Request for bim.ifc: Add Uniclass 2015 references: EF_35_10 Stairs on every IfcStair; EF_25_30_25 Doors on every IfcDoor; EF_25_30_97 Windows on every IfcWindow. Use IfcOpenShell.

First a look at what the model holds.

```python
import ifcopenshell

model = ifcopenshell.open("bim.ifc")
print(model.schema)
print("classifications:", [c.Name for c in model.by_type("IfcClassification")])
for ifc_class in ("IfcDoor", "IfcRoof", "IfcStair", "IfcWall", "IfcWindow"):
    print(ifc_class, len(model.by_type(ifc_class)))
```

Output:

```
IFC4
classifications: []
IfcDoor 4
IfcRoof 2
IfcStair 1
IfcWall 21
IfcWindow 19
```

```python
import ifcopenshell
import ifcopenshell.api.classification

model = ifcopenshell.open("bim.ifc")

system = ifcopenshell.api.classification.add_classification(model, classification="Uniclass 2015")

codes = {
    "IfcStair": ("EF_35_10", "Stairs"),
    "IfcDoor": ("EF_25_30_25", "Doors"),
    "IfcWindow": ("EF_25_30_97", "Windows"),
}
for ifc_class, (code, name) in codes.items():
    products = model.by_type(ifc_class)
    ifcopenshell.api.classification.add_reference(
        model, products=products, classification=system, identification=code, name=name
    )
    print(code, len(products))

model.write("bim_edited.ifc")
```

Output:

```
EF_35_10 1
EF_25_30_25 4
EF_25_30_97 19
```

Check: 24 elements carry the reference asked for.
